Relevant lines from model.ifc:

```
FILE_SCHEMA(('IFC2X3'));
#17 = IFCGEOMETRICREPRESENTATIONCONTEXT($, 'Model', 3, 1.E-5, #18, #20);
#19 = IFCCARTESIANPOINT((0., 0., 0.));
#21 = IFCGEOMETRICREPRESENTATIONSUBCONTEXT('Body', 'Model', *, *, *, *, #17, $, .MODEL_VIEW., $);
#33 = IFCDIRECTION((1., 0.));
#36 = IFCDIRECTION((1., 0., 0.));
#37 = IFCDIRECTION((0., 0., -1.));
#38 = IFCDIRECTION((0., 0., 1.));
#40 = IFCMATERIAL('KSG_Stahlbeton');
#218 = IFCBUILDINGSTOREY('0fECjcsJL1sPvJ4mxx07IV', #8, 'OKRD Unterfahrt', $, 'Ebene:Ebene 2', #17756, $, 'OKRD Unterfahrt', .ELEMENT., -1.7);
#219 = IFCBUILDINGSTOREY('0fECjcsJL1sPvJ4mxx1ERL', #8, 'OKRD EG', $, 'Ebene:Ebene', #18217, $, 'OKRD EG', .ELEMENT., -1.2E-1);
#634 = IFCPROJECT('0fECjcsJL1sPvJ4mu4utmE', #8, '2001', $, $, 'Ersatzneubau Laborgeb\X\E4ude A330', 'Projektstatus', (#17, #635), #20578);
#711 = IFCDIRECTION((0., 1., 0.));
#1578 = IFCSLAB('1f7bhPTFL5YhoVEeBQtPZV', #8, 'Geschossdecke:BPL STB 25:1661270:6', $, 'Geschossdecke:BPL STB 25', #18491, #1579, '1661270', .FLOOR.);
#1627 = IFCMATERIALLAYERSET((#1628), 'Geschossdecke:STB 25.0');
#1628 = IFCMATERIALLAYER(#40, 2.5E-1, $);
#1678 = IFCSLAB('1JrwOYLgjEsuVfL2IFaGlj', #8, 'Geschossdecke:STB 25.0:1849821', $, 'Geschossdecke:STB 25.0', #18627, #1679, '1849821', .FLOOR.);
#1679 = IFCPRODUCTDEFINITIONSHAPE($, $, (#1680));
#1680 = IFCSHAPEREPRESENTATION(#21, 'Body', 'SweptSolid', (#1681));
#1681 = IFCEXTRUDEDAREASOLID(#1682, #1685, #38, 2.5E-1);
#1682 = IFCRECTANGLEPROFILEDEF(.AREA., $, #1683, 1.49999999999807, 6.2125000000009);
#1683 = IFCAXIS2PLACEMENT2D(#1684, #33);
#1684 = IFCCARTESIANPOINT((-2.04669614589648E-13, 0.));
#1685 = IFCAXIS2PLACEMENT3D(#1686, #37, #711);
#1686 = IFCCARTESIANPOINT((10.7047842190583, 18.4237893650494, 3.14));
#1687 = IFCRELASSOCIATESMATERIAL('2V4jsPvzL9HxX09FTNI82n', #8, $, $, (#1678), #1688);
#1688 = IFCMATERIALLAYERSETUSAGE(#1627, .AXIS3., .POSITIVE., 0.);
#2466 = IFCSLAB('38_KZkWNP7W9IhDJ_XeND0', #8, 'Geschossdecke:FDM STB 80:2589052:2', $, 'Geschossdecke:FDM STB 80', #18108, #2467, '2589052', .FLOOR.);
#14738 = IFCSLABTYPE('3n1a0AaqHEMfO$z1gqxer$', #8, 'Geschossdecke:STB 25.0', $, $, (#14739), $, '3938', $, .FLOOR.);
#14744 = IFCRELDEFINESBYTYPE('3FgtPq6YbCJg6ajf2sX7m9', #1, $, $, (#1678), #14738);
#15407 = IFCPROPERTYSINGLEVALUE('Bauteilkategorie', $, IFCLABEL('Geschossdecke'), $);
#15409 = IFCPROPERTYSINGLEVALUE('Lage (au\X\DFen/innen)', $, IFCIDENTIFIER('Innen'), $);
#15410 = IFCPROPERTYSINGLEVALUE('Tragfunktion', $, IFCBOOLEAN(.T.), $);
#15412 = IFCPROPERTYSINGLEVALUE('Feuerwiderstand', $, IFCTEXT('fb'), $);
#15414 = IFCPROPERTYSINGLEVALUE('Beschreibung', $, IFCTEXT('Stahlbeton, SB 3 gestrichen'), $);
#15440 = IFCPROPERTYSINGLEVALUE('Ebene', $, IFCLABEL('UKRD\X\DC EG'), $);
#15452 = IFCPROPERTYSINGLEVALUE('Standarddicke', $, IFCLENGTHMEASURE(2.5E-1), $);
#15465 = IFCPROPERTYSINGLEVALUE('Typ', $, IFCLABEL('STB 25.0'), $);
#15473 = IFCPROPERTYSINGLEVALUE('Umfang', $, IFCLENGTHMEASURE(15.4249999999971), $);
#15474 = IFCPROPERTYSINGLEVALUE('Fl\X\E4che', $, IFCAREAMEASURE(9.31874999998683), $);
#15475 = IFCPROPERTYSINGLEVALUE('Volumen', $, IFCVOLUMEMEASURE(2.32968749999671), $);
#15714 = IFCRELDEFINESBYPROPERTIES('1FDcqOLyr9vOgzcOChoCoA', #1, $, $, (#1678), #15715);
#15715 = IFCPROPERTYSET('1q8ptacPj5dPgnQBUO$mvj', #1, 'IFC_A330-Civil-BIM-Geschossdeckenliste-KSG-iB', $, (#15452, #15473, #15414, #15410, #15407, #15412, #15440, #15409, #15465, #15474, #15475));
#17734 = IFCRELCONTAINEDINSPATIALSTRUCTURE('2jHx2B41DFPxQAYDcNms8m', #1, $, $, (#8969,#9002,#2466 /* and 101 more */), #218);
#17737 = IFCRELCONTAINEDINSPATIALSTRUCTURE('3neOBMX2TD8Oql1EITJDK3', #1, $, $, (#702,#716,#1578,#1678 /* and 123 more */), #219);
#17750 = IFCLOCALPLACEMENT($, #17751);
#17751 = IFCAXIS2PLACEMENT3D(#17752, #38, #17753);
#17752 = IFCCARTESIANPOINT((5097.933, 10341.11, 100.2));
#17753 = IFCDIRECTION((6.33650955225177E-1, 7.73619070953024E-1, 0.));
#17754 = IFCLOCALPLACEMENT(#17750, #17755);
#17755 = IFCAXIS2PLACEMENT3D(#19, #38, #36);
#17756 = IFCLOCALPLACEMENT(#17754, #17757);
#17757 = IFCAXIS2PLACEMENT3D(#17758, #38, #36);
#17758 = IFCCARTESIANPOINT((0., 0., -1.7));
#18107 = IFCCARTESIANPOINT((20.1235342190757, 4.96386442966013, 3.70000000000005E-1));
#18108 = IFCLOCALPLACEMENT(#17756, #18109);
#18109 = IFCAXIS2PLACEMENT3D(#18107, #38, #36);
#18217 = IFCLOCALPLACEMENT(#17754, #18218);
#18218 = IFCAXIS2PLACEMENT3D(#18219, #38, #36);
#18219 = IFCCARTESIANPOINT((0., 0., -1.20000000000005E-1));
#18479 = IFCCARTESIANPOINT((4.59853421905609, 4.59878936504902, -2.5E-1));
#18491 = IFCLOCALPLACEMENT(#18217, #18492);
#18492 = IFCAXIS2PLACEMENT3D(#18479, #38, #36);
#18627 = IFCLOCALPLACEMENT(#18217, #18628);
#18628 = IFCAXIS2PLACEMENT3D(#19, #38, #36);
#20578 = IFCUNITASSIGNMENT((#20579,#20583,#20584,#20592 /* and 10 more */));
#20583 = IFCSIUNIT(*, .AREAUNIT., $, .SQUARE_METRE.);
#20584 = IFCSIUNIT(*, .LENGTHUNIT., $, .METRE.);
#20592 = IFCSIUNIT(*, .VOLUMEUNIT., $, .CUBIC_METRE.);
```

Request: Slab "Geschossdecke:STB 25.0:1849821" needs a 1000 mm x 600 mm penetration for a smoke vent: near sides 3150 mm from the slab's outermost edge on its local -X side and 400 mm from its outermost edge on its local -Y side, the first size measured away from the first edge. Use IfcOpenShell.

```python
import numpy as np
import ifcopenshell
import ifcopenshell.api.feature
import ifcopenshell.api.geometry
import ifcopenshell.api.pset
import ifcopenshell.api.root
import ifcopenshell.geom
import ifcopenshell.util.element
import ifcopenshell.util.placement
import ifcopenshell.util.representation
import ifcopenshell.util.shape
import ifcopenshell.util.unit

model = ifcopenshell.open("model.ifc")
unit_scale = ifcopenshell.util.unit.calculate_unit_scale(model)
area_scale = ifcopenshell.util.unit.calculate_unit_scale(model, "AREAUNIT")
volume_scale = ifcopenshell.util.unit.calculate_unit_scale(model, "VOLUMEUNIT")
settings = ifcopenshell.geom.settings()


def volume(element):
    """Net volume in cubic metres, openings subtracted."""
    shape = ifcopenshell.geom.create_shape(settings, element)
    return ifcopenshell.util.shape.get_volume(shape.geometry)


slab = model.by_guid("1JrwOYLgjEsuVfL2IFaGlj")
before = volume(slab)

# Extent in the slab's own axes, in metres. The edges named are its -X and -Y sides.
slab_shape = ifcopenshell.geom.create_shape(settings, slab)
vertices = ifcopenshell.util.shape.get_vertices(slab_shape.geometry)
x_min, y_min, bottom = vertices.min(axis=0)
top = vertices[:, 2].max()

opening = ifcopenshell.api.root.create_entity(model, ifc_class="IfcOpeningElement", name="Smoke vent opening")
context = ifcopenshell.util.representation.get_context(model, "Model", "Body", "MODEL_VIEW")
width, depth = 1, 0.6
outline = [(0.0, 0.0), (width, 0.0), (width, depth), (0.0, depth), (0.0, 0.0)]
# Overshoot both faces by 50 mm so the cut is clean.
shape = ifcopenshell.api.geometry.add_slab_representation(
    model, context=context, depth=top - bottom + 0.1, polyline=outline
)
ifcopenshell.api.geometry.assign_representation(model, product=opening, representation=shape)

matrix = ifcopenshell.util.placement.get_local_placement(slab.ObjectPlacement)
matrix[:, 3] = matrix @ np.append(np.array([x_min + 3.15, y_min + 0.4, bottom - 0.05]) / unit_scale, 1.0)
ifcopenshell.api.geometry.edit_object_placement(model, product=opening, matrix=matrix, is_si=False)
ifcopenshell.api.feature.add_feature(model, feature=opening, element=slab)

after = volume(slab)

# Update the slab's stored quantities.
pset = model.by_id(ifcopenshell.util.element.get_pset(slab, "IFC_A330-Civil-BIM-Geschossdeckenliste-KSG-iB", should_inherit=False)["id"])
ifcopenshell.api.pset.edit_pset(model, pset=pset, properties={
    "Fläche": model.create_entity("IfcAreaMeasure", after / (top - bottom) / area_scale),
    "Volumen": model.create_entity("IfcVolumeMeasure", after / volume_scale),
})

print(f"slab volume {before:.3f} -> {after:.3f} m3")

model.write("model_v2.ifc")
```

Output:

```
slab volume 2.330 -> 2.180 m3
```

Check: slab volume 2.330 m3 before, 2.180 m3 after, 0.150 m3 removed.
